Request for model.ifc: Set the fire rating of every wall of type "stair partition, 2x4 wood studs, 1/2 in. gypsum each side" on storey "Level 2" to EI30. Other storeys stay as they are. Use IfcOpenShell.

First a look at what the model holds.

```python
import ifcopenshell
import ifcopenshell.util.element

model = ifcopenshell.open("model.ifc")
print(model.schema)
storey = next(s for s in model.by_type("IfcBuildingStorey") if s.Name == "Level 2")
walls = [e for e in ifcopenshell.util.element.get_decomposition(storey) if e.is_a("IfcWall")]
seen = {}
for e in walls:
    element_type = ifcopenshell.util.element.get_type(e)
    key = (element_type.Name if element_type != e and element_type else None, ifcopenshell.util.element.get_pset(e, "Pset_WallCommon", "FireRating"))
    seen[key] = seen.get(key, 0) + 1
for (name, value), count in sorted(seen.items(), key=str):
    print(count, "x", name, "|", value)
```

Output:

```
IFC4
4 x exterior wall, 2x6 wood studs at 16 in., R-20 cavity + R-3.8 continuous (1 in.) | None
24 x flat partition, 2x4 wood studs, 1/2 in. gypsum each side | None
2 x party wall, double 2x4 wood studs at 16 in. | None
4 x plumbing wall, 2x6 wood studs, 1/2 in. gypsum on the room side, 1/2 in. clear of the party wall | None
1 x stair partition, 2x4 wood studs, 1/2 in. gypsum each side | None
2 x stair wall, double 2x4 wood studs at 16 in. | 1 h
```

```python
import ifcopenshell
import ifcopenshell.api.pset
import ifcopenshell.util.element

model = ifcopenshell.open("model.ifc")

storey = next(s for s in model.by_type("IfcBuildingStorey") if s.Name == "Level 2")
walls = [e for e in ifcopenshell.util.element.get_decomposition(storey) if e.is_a("IfcWall")]

count = 0
for e in walls:
    element_type = ifcopenshell.util.element.get_type(e)
    if element_type in (None, e) or element_type.Name != "stair partition, 2x4 wood studs, 1/2 in. gypsum each side":
        continue
    # add_pset returns the element's existing set when there is one.
    pset = ifcopenshell.api.pset.add_pset(model, product=e, name="Pset_WallCommon")
    ifcopenshell.api.pset.edit_pset(model, pset=pset, properties={"FireRating": "EI30"})
    count += 1

print(count, "walls updated")

model.write("model_rev.ifc")
```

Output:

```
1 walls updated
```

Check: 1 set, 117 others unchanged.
